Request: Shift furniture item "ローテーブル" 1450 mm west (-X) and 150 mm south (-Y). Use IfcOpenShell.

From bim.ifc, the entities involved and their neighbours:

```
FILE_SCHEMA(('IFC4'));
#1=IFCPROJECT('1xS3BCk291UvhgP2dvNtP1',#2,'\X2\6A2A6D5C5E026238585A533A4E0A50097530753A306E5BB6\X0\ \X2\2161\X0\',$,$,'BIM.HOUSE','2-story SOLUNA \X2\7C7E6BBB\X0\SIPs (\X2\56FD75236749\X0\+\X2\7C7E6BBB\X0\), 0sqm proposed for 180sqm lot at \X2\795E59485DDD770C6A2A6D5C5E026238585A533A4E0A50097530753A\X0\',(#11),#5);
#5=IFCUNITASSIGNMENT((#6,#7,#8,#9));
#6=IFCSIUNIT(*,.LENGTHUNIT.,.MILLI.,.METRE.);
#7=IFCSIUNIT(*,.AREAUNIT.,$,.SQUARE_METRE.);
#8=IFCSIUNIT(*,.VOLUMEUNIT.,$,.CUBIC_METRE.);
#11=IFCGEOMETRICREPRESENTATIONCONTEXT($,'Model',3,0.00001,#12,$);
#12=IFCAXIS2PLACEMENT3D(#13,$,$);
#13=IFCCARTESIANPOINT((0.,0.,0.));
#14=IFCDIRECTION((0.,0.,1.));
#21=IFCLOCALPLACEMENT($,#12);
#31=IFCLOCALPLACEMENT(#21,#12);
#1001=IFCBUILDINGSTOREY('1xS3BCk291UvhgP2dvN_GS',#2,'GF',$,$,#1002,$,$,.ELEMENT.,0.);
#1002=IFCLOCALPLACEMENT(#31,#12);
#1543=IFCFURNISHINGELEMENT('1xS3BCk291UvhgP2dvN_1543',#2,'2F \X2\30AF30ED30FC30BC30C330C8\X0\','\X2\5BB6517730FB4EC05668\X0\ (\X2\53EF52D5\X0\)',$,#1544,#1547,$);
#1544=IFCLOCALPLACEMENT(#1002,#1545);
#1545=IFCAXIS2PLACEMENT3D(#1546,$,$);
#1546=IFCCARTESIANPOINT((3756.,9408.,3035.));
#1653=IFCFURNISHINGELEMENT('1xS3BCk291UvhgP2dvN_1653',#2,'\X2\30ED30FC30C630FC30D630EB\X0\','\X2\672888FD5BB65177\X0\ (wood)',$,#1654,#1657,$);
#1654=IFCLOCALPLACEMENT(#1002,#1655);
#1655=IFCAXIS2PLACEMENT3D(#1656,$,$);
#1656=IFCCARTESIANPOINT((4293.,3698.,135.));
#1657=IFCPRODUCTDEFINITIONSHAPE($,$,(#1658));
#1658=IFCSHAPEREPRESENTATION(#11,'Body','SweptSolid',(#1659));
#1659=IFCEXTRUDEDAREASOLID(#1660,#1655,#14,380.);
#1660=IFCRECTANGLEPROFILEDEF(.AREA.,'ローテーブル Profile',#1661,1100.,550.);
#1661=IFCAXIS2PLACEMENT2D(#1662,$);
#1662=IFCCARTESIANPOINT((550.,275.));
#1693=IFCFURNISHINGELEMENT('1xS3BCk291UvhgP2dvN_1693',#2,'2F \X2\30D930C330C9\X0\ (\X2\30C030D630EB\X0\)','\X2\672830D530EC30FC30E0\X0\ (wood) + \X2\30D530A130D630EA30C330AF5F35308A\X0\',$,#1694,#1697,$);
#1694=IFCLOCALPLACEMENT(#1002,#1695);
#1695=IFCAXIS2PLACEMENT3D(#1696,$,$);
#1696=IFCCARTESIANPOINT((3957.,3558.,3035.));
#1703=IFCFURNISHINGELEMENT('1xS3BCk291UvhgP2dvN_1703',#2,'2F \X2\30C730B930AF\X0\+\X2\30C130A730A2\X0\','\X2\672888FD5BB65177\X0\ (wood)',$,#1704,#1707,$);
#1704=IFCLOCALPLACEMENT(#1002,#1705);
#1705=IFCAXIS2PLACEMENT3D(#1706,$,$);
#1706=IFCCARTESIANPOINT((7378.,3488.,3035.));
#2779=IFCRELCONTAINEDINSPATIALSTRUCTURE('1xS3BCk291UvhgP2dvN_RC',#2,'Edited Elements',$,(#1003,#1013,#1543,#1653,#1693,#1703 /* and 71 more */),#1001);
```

```python
import ifcopenshell
import ifcopenshell.api.geometry
import ifcopenshell.util.placement
import ifcopenshell.util.unit

model = ifcopenshell.open("bim.ifc")
unit_scale = ifcopenshell.util.unit.calculate_unit_scale(model)

item = model.by_guid("1xS3BCk291UvhgP2dvN_1653")
matrix = ifcopenshell.util.placement.get_local_placement(item.ObjectPlacement)
matrix[0, 3] -= 1.45 / unit_scale
matrix[1, 3] -= 0.15 / unit_scale
ifcopenshell.api.geometry.edit_object_placement(model, product=item, matrix=matrix, is_si=False)

print(ifcopenshell.util.placement.get_local_placement(item.ObjectPlacement).round(3) + 0.0)

model.write("bim_updated.ifc")
```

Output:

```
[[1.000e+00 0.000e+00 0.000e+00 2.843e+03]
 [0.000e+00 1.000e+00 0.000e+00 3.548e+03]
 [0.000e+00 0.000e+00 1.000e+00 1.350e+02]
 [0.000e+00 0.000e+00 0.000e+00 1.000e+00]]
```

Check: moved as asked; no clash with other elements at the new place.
